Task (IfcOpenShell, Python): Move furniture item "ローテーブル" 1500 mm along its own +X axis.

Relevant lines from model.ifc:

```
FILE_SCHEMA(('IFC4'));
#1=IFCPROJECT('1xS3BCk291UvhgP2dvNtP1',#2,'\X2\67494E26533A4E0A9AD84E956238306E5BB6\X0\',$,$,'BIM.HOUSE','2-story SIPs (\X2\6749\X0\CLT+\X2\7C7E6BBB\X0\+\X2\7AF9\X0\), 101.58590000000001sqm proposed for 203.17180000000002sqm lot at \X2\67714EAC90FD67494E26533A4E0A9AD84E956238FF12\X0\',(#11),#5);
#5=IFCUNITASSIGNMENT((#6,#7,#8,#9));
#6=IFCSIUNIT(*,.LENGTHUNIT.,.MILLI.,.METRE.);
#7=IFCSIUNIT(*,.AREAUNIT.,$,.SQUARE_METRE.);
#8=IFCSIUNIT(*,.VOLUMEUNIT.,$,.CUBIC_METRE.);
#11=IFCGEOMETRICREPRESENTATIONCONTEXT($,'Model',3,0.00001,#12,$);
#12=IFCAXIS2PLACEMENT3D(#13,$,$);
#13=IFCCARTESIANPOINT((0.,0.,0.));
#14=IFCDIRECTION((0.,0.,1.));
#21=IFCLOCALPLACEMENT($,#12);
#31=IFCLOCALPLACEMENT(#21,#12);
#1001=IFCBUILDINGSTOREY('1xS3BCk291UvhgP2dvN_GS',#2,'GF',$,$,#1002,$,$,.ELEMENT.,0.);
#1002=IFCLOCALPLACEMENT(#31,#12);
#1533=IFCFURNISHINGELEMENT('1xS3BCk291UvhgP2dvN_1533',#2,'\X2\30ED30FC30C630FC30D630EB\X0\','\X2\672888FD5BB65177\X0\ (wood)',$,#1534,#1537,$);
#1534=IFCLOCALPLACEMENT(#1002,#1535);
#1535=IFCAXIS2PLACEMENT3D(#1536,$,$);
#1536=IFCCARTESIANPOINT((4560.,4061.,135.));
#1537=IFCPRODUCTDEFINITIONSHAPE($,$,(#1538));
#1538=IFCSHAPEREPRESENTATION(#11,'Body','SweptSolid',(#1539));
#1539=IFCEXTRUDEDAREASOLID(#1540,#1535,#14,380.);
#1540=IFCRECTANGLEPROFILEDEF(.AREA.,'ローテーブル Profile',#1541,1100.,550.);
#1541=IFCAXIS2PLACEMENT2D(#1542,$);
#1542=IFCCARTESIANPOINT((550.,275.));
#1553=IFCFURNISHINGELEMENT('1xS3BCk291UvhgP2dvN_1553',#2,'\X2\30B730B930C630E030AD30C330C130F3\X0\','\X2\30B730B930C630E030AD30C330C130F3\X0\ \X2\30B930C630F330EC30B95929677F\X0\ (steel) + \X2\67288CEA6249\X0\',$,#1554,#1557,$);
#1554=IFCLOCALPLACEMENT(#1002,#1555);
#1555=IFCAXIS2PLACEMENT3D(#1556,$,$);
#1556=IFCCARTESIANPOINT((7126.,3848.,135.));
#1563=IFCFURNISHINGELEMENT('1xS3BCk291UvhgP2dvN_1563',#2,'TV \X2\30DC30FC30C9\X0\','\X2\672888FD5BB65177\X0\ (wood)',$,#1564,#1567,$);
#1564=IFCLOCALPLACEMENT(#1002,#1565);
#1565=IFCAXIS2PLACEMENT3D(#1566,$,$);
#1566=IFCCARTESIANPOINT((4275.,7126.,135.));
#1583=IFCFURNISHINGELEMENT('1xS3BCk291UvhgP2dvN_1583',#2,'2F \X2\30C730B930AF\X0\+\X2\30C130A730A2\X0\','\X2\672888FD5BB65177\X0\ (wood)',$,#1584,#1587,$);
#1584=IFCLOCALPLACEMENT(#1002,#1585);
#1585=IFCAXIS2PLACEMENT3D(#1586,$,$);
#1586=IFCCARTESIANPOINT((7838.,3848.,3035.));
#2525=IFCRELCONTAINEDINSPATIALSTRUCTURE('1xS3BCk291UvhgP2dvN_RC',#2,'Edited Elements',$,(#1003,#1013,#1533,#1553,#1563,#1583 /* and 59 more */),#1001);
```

```python
import ifcopenshell
import ifcopenshell.api.geometry
import ifcopenshell.util.placement

model = ifcopenshell.open("model.ifc")

item = model.by_guid("1xS3BCk291UvhgP2dvN_1533")
matrix = ifcopenshell.util.placement.get_local_placement(item.ObjectPlacement)
matrix[:3, 3] += matrix[:3, 0] * 1500.0
ifcopenshell.api.geometry.edit_object_placement(model, product=item, matrix=matrix, is_si=False)

print(ifcopenshell.util.placement.get_local_placement(item.ObjectPlacement).round(3) + 0.0)

model.write("model_updated.ifc")
```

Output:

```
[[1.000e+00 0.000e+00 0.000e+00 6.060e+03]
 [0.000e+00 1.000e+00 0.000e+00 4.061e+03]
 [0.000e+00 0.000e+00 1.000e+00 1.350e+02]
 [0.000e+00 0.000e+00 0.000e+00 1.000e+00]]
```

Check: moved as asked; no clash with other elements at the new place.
